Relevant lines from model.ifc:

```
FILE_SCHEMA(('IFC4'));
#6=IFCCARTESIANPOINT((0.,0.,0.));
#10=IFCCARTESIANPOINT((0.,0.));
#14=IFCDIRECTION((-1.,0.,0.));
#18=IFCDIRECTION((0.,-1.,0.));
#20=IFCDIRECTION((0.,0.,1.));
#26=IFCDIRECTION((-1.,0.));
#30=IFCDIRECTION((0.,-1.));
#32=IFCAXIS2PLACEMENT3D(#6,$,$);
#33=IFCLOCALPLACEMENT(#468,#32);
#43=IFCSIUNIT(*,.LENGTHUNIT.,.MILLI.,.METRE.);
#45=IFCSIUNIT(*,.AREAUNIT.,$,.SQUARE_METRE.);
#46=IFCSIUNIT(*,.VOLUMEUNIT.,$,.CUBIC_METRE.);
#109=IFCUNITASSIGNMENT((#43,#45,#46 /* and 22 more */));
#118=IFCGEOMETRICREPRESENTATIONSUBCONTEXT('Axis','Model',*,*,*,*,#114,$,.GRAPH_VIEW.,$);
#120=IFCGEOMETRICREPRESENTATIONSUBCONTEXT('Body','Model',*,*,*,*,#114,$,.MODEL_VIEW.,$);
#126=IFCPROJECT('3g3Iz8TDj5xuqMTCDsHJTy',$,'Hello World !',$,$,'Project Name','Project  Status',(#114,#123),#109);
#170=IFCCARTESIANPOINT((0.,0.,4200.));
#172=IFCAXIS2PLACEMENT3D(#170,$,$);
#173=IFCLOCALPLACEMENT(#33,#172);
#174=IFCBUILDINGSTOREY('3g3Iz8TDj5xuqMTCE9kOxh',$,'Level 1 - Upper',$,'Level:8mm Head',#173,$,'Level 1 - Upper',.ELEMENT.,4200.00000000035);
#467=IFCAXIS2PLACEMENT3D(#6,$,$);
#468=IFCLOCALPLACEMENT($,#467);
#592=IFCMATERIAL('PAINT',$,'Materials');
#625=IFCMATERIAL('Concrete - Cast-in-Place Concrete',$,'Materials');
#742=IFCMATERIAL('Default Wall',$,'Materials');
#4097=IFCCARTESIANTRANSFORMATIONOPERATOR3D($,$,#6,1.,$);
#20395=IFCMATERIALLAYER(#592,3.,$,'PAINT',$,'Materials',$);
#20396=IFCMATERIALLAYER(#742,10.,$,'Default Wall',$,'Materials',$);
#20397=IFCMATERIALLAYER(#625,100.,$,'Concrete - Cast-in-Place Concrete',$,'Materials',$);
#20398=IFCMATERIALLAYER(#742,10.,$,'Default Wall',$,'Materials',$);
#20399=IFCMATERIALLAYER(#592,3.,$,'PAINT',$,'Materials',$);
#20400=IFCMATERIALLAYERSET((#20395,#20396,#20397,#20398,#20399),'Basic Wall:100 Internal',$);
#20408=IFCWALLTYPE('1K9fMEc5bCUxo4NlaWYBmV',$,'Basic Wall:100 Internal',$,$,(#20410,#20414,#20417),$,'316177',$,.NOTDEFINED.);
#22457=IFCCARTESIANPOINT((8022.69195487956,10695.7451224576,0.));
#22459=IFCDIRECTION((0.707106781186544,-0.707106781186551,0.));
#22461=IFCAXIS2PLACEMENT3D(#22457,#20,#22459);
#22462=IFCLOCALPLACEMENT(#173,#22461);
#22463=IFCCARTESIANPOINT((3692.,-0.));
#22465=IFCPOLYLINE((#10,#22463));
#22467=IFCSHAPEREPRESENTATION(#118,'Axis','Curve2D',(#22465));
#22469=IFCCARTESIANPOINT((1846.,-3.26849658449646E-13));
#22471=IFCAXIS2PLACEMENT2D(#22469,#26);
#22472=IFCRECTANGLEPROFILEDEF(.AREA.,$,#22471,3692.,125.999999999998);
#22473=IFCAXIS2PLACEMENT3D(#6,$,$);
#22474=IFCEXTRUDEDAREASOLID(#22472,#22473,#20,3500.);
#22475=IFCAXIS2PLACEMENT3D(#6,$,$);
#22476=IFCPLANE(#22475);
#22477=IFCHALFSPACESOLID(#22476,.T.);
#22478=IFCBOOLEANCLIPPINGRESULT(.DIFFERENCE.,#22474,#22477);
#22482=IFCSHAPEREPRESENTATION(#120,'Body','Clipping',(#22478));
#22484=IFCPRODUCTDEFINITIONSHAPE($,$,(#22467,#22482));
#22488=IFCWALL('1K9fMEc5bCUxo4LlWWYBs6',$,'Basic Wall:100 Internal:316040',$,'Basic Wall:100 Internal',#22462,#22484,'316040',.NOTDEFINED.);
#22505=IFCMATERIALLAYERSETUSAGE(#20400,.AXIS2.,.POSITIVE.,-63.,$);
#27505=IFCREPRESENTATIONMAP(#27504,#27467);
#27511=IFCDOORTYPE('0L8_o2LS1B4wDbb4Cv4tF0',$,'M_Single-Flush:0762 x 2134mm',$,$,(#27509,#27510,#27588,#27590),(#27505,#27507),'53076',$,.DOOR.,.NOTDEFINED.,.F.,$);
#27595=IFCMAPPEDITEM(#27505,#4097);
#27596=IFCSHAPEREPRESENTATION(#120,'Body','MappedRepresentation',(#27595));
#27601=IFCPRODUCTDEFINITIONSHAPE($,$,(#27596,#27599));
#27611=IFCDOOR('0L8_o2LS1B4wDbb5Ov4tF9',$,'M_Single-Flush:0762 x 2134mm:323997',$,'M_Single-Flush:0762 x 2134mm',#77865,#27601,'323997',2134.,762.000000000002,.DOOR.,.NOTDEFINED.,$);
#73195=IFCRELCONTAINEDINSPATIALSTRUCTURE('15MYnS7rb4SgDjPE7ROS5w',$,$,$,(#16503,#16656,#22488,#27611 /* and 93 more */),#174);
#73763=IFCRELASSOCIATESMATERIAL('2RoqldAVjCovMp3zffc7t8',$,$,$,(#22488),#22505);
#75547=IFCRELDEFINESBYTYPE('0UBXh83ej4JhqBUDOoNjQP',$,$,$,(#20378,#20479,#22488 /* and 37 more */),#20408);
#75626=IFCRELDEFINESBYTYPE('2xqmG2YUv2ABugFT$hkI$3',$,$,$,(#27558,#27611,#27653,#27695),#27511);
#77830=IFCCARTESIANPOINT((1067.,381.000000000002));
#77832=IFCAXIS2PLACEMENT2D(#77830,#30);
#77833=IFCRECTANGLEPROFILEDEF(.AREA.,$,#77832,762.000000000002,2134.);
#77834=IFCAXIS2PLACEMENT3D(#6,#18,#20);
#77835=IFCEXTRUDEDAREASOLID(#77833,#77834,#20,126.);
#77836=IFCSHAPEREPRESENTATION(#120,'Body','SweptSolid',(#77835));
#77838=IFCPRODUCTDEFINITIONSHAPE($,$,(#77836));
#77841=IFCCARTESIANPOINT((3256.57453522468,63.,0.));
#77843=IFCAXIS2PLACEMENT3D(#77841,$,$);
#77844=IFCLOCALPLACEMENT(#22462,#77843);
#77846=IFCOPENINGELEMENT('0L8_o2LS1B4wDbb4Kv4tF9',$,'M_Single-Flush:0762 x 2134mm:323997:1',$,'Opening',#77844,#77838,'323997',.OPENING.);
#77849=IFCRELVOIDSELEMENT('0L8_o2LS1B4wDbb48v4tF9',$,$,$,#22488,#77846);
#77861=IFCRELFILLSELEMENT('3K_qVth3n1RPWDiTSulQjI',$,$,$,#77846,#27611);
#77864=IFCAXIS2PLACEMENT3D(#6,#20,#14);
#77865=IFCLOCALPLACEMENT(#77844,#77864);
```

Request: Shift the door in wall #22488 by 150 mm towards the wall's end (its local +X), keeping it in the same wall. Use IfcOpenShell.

```python
import ifcopenshell
import ifcopenshell.api.geometry
import ifcopenshell.util.placement
import ifcopenshell.util.unit

model = ifcopenshell.open("model.ifc")
unit_scale = ifcopenshell.util.unit.calculate_unit_scale(model)

door = model.by_guid("0L8_o2LS1B4wDbb5Ov4tF9")
opening = door.FillsVoids[0].RelatingOpeningElement
wall = opening.VoidsElements[0].RelatingBuildingElement

wall_matrix = ifcopenshell.util.placement.get_local_placement(wall.ObjectPlacement)
shift = wall_matrix[:3, 0] * 0.15 / unit_scale
before = ifcopenshell.util.placement.get_local_placement(door.ObjectPlacement)[:3, 3].copy()

# The door is placed relative to its opening, so it follows when the opening moves.
matrix = ifcopenshell.util.placement.get_local_placement(opening.ObjectPlacement)
matrix[:3, 3] += shift
ifcopenshell.api.geometry.edit_object_placement(
    model, product=opening, matrix=matrix, is_si=False, should_transform_children=True
)

after = ifcopenshell.util.placement.get_local_placement(door.ObjectPlacement)[:3, 3]
print("door moved by", (after - before).round(3) + 0.0)

model.write("model_v2.ifc")
```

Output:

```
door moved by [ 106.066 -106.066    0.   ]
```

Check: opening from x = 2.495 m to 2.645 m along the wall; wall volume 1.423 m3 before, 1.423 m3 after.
